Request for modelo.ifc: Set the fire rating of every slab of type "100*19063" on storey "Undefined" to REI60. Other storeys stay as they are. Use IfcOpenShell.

First a look at what the model holds.

```python
import ifcopenshell
import ifcopenshell.util.element

model = ifcopenshell.open("modelo.ifc")
print(model.schema)
storey = next(s for s in model.by_type("IfcBuildingStorey") if s.Name == "Undefined")
slabs = [e for e in ifcopenshell.util.element.get_decomposition(storey) if e.is_a("IfcSlab")]
seen = {}
for e in slabs:
    element_type = ifcopenshell.util.element.get_type(e)
    key = (element_type.Name if element_type != e and element_type else None, ifcopenshell.util.element.get_pset(e, "Pset_SlabCommon", "FireRating"))
    seen[key] = seen.get(key, 0) + 1
for (name, value), count in sorted(seen.items(), key=str):
    print(count, "x", name, "|", value)
```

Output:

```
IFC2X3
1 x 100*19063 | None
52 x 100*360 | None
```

```python
import ifcopenshell
import ifcopenshell.api.pset
import ifcopenshell.util.element

model = ifcopenshell.open("modelo.ifc")

storey = next(s for s in model.by_type("IfcBuildingStorey") if s.Name == "Undefined")
slabs = [e for e in ifcopenshell.util.element.get_decomposition(storey) if e.is_a("IfcSlab")]

count = 0
for e in slabs:
    element_type = ifcopenshell.util.element.get_type(e)
    if element_type in (None, e) or element_type.Name != "100*19063":
        continue
    found = ifcopenshell.util.element.get_pset(e, "Pset_SlabCommon", should_inherit=False)
    if found:
        pset = model.by_id(found["id"])
        if len(ifcopenshell.util.element.get_elements_by_pset(pset)) > 1:
            pset = ifcopenshell.api.pset.unshare_pset(model, products=[e], pset=pset)[0]
    else:
        pset = ifcopenshell.api.pset.add_pset(model, product=e, name="Pset_SlabCommon")
    ifcopenshell.api.pset.edit_pset(model, pset=pset, properties={"FireRating": "REI60"})
    count += 1

print(count, "slabs updated")

model.write("modelo_rev.ifc")
```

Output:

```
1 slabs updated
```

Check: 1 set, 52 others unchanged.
